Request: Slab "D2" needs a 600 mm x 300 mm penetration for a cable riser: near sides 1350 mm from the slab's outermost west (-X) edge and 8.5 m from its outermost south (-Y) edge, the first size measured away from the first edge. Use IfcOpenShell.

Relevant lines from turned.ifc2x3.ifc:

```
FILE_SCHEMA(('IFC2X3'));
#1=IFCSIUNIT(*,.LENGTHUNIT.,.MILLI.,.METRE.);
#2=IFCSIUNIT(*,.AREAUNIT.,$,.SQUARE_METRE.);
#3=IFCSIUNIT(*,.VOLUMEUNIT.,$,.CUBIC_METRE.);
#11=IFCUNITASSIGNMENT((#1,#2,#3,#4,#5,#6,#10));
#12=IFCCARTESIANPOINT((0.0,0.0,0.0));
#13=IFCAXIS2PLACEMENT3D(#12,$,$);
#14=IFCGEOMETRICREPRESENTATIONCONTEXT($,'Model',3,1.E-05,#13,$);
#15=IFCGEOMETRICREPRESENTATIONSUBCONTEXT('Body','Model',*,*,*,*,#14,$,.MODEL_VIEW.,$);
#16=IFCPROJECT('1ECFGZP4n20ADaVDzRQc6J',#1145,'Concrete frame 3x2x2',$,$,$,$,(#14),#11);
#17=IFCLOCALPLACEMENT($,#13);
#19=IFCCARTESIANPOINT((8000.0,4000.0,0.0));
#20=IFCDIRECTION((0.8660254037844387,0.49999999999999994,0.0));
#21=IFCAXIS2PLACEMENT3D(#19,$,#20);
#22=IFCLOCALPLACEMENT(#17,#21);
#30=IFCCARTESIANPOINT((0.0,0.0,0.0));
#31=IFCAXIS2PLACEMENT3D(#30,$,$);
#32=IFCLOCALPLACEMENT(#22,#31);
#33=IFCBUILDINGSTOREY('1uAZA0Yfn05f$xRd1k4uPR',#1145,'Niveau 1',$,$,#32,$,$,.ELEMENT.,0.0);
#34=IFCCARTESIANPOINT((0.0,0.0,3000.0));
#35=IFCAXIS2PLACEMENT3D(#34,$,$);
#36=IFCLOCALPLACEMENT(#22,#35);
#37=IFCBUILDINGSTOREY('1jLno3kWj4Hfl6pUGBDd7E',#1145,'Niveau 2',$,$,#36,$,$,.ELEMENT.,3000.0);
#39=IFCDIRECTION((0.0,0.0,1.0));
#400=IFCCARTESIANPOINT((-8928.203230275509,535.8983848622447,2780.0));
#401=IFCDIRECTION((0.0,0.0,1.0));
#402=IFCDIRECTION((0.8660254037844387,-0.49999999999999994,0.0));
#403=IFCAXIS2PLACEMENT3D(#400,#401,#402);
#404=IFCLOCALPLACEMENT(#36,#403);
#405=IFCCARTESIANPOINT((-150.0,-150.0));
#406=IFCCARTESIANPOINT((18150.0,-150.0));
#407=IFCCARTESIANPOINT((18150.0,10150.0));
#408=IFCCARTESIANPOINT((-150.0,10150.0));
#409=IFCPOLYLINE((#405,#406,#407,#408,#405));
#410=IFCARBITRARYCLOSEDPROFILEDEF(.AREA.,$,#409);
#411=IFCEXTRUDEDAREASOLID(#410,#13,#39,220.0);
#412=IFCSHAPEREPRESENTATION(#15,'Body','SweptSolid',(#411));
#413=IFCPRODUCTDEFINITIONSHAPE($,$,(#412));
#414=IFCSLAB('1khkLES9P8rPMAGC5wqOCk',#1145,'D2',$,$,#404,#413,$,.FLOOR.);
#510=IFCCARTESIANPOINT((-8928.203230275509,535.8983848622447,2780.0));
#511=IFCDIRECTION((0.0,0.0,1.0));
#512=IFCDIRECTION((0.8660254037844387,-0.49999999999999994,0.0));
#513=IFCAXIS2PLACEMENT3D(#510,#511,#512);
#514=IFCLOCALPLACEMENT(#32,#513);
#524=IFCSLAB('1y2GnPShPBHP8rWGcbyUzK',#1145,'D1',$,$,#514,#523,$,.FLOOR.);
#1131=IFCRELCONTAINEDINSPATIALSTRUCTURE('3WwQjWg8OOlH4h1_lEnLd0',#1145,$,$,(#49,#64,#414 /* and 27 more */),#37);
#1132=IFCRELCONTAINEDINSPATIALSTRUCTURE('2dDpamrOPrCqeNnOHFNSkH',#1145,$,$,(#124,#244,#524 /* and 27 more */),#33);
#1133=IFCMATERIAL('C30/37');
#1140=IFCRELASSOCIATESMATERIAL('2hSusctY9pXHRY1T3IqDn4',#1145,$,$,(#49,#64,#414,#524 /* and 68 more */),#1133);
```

```python
import numpy as np
import ifcopenshell
import ifcopenshell.api.feature
import ifcopenshell.api.geometry
import ifcopenshell.api.root
import ifcopenshell.geom
import ifcopenshell.util.placement
import ifcopenshell.util.representation
import ifcopenshell.util.shape
import ifcopenshell.util.unit

model = ifcopenshell.open("turned.ifc2x3.ifc")
unit_scale = ifcopenshell.util.unit.calculate_unit_scale(model)
settings = ifcopenshell.geom.settings()


def volume(element):
    """Net volume in cubic metres, openings subtracted."""
    shape = ifcopenshell.geom.create_shape(settings, element)
    return ifcopenshell.util.shape.get_volume(shape.geometry)


slab = model.by_guid("1khkLES9P8rPMAGC5wqOCk")
before = volume(slab)

# Extent in the slab's own axes, in metres. The edges named are its -X and -Y sides.
slab_shape = ifcopenshell.geom.create_shape(settings, slab)
vertices = ifcopenshell.util.shape.get_vertices(slab_shape.geometry)
x_min, y_min, bottom = vertices.min(axis=0)
top = vertices[:, 2].max()

opening = ifcopenshell.api.root.create_entity(model, ifc_class="IfcOpeningElement", name="Cable riser opening")
context = ifcopenshell.util.representation.get_context(model, "Model", "Body", "MODEL_VIEW")
width, depth = 0.6, 0.3
outline = [(0.0, 0.0), (width, 0.0), (width, depth), (0.0, depth), (0.0, 0.0)]
# Overshoot both faces by 50 mm so the cut is clean.
shape = ifcopenshell.api.geometry.add_slab_representation(
    model, context=context, depth=top - bottom + 0.1, polyline=outline
)
ifcopenshell.api.geometry.assign_representation(model, product=opening, representation=shape)

matrix = ifcopenshell.util.placement.get_local_placement(slab.ObjectPlacement)
matrix[:, 3] = matrix @ np.append(np.array([x_min + 1.35, y_min + 8.5, bottom - 0.05]) / unit_scale, 1.0)
ifcopenshell.api.geometry.edit_object_placement(model, product=opening, matrix=matrix, is_si=False)
ifcopenshell.api.feature.add_feature(model, feature=opening, element=slab)

after = volume(slab)

print(f"slab volume {before:.3f} -> {after:.3f} m3")

model.write("turned.ifc2x3_v2.ifc")
```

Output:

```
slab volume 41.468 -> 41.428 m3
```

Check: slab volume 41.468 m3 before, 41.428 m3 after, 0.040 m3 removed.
